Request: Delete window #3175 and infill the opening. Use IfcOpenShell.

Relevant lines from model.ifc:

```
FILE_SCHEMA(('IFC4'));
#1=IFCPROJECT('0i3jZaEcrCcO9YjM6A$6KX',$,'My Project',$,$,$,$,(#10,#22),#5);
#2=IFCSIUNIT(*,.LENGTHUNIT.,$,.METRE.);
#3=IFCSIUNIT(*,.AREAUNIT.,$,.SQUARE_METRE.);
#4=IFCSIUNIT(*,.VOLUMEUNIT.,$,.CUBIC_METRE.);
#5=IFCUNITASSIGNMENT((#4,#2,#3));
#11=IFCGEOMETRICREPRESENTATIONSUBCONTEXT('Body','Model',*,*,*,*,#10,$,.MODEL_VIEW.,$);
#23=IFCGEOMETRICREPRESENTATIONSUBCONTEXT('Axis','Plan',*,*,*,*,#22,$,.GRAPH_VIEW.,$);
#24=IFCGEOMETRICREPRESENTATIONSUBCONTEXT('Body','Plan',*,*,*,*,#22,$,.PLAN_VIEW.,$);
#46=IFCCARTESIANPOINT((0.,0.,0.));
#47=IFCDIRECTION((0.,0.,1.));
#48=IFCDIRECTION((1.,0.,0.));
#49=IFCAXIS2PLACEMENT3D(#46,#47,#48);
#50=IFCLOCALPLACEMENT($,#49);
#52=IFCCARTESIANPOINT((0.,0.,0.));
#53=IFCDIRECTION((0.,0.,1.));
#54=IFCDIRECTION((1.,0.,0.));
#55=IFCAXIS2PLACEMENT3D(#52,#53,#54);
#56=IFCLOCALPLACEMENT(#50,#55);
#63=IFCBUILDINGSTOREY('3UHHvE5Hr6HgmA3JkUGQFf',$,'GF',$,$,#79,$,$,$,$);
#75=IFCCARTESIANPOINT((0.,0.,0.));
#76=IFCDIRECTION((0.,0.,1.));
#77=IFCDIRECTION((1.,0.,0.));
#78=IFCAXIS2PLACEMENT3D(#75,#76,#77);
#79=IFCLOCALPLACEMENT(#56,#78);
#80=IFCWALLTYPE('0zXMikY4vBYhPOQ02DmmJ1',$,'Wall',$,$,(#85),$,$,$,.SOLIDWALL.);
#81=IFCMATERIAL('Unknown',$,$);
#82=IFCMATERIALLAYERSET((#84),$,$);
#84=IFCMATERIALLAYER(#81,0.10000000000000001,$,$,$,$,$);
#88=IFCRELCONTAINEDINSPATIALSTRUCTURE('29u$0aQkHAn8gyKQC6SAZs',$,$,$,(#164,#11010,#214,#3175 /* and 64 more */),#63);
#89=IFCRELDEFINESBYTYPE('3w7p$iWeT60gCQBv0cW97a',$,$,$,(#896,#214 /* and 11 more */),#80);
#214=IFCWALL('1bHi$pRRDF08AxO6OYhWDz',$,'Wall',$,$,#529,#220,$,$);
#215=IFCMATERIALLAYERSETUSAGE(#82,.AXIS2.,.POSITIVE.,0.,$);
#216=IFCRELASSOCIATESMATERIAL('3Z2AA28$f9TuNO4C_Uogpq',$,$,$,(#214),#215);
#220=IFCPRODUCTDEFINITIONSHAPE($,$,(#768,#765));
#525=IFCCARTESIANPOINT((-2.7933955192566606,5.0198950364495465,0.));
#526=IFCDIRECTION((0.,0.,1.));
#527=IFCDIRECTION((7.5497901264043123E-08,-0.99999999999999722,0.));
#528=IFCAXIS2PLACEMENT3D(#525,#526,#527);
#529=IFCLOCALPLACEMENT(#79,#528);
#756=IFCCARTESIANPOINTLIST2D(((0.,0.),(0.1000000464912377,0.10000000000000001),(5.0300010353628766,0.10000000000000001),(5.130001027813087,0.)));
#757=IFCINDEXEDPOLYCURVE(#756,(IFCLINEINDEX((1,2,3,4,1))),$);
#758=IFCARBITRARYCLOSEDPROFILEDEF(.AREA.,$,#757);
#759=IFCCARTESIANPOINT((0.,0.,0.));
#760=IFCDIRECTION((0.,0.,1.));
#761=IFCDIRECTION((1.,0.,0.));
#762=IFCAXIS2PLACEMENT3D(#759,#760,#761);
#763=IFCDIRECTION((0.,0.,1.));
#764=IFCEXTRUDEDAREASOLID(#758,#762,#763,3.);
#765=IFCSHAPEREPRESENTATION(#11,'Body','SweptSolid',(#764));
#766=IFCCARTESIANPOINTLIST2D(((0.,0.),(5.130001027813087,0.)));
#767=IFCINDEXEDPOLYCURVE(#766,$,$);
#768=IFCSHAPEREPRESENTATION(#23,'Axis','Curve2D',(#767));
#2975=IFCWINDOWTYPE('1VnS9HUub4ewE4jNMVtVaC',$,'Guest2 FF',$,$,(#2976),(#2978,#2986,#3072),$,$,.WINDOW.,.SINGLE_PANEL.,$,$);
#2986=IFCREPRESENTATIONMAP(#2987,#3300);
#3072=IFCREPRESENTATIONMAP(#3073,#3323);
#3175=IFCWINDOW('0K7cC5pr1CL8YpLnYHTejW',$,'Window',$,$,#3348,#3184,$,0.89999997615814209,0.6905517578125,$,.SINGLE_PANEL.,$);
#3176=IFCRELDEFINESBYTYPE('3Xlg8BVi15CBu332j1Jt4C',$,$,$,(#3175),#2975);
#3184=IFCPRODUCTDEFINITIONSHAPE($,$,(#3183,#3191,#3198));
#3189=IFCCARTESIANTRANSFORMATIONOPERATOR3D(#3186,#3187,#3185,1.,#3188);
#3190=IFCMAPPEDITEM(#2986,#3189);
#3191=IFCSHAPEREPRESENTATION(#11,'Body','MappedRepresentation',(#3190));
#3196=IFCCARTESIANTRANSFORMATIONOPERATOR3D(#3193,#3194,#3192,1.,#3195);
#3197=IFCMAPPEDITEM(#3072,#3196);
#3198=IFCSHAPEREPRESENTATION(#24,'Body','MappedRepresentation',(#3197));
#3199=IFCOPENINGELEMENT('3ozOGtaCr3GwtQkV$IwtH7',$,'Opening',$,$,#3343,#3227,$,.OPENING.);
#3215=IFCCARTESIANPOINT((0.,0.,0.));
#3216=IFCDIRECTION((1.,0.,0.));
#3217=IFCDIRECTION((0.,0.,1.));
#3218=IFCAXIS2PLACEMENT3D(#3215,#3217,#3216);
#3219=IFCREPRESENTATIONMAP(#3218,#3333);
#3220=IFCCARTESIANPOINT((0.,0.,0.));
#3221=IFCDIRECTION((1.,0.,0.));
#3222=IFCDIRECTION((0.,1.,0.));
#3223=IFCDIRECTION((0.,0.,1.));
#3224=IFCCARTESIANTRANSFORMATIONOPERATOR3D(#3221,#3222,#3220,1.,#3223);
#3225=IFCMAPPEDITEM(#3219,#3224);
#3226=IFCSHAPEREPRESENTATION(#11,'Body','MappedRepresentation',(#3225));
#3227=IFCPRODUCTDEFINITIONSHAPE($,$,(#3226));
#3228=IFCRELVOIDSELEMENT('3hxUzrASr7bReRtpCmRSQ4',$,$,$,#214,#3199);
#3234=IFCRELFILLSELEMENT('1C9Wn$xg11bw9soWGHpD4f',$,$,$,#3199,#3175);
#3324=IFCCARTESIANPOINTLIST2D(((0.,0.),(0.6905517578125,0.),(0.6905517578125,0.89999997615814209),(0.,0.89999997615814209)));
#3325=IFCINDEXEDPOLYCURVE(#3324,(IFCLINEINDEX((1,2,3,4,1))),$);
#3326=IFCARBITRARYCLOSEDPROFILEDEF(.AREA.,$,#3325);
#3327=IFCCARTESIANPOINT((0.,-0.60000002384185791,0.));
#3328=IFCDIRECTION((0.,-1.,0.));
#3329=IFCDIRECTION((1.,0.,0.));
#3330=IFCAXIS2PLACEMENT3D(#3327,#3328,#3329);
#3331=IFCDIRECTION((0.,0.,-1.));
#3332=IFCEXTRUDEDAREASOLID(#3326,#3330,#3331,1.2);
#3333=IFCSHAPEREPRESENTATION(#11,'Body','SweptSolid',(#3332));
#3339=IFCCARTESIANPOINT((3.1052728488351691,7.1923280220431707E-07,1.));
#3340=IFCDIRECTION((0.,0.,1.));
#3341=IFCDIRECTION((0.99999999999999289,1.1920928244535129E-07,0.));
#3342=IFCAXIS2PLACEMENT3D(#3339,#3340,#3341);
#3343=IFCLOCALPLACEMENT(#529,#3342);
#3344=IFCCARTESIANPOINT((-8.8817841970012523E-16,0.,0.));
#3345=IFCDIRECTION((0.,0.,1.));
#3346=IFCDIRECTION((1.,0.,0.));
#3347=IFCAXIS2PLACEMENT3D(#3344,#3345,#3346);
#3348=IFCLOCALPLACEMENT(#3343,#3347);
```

```python
import ifcopenshell
import ifcopenshell.api.feature
import ifcopenshell.api.root
import ifcopenshell.geom
import ifcopenshell.util.shape

model = ifcopenshell.open("model.ifc")
settings = ifcopenshell.geom.settings()


def volume(element):
    """Net volume in cubic metres, openings subtracted."""
    shape = ifcopenshell.geom.create_shape(settings, element)
    return ifcopenshell.util.shape.get_volume(shape.geometry)


window = model.by_guid("0K7cC5pr1CL8YpLnYHTejW")
opening = window.FillsVoids[0].RelatingOpeningElement
wall = opening.VoidsElements[0].RelatingBuildingElement
before = volume(wall)

ifcopenshell.api.root.remove_product(model, product=window)
ifcopenshell.api.feature.remove_feature(model, feature=opening)

after = volume(wall)

print(f"wall volume {before:.3f} -> {after:.3f} m3")

model.write("model_rev.ifc")
```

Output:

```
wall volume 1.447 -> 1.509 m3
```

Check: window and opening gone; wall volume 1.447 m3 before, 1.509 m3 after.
